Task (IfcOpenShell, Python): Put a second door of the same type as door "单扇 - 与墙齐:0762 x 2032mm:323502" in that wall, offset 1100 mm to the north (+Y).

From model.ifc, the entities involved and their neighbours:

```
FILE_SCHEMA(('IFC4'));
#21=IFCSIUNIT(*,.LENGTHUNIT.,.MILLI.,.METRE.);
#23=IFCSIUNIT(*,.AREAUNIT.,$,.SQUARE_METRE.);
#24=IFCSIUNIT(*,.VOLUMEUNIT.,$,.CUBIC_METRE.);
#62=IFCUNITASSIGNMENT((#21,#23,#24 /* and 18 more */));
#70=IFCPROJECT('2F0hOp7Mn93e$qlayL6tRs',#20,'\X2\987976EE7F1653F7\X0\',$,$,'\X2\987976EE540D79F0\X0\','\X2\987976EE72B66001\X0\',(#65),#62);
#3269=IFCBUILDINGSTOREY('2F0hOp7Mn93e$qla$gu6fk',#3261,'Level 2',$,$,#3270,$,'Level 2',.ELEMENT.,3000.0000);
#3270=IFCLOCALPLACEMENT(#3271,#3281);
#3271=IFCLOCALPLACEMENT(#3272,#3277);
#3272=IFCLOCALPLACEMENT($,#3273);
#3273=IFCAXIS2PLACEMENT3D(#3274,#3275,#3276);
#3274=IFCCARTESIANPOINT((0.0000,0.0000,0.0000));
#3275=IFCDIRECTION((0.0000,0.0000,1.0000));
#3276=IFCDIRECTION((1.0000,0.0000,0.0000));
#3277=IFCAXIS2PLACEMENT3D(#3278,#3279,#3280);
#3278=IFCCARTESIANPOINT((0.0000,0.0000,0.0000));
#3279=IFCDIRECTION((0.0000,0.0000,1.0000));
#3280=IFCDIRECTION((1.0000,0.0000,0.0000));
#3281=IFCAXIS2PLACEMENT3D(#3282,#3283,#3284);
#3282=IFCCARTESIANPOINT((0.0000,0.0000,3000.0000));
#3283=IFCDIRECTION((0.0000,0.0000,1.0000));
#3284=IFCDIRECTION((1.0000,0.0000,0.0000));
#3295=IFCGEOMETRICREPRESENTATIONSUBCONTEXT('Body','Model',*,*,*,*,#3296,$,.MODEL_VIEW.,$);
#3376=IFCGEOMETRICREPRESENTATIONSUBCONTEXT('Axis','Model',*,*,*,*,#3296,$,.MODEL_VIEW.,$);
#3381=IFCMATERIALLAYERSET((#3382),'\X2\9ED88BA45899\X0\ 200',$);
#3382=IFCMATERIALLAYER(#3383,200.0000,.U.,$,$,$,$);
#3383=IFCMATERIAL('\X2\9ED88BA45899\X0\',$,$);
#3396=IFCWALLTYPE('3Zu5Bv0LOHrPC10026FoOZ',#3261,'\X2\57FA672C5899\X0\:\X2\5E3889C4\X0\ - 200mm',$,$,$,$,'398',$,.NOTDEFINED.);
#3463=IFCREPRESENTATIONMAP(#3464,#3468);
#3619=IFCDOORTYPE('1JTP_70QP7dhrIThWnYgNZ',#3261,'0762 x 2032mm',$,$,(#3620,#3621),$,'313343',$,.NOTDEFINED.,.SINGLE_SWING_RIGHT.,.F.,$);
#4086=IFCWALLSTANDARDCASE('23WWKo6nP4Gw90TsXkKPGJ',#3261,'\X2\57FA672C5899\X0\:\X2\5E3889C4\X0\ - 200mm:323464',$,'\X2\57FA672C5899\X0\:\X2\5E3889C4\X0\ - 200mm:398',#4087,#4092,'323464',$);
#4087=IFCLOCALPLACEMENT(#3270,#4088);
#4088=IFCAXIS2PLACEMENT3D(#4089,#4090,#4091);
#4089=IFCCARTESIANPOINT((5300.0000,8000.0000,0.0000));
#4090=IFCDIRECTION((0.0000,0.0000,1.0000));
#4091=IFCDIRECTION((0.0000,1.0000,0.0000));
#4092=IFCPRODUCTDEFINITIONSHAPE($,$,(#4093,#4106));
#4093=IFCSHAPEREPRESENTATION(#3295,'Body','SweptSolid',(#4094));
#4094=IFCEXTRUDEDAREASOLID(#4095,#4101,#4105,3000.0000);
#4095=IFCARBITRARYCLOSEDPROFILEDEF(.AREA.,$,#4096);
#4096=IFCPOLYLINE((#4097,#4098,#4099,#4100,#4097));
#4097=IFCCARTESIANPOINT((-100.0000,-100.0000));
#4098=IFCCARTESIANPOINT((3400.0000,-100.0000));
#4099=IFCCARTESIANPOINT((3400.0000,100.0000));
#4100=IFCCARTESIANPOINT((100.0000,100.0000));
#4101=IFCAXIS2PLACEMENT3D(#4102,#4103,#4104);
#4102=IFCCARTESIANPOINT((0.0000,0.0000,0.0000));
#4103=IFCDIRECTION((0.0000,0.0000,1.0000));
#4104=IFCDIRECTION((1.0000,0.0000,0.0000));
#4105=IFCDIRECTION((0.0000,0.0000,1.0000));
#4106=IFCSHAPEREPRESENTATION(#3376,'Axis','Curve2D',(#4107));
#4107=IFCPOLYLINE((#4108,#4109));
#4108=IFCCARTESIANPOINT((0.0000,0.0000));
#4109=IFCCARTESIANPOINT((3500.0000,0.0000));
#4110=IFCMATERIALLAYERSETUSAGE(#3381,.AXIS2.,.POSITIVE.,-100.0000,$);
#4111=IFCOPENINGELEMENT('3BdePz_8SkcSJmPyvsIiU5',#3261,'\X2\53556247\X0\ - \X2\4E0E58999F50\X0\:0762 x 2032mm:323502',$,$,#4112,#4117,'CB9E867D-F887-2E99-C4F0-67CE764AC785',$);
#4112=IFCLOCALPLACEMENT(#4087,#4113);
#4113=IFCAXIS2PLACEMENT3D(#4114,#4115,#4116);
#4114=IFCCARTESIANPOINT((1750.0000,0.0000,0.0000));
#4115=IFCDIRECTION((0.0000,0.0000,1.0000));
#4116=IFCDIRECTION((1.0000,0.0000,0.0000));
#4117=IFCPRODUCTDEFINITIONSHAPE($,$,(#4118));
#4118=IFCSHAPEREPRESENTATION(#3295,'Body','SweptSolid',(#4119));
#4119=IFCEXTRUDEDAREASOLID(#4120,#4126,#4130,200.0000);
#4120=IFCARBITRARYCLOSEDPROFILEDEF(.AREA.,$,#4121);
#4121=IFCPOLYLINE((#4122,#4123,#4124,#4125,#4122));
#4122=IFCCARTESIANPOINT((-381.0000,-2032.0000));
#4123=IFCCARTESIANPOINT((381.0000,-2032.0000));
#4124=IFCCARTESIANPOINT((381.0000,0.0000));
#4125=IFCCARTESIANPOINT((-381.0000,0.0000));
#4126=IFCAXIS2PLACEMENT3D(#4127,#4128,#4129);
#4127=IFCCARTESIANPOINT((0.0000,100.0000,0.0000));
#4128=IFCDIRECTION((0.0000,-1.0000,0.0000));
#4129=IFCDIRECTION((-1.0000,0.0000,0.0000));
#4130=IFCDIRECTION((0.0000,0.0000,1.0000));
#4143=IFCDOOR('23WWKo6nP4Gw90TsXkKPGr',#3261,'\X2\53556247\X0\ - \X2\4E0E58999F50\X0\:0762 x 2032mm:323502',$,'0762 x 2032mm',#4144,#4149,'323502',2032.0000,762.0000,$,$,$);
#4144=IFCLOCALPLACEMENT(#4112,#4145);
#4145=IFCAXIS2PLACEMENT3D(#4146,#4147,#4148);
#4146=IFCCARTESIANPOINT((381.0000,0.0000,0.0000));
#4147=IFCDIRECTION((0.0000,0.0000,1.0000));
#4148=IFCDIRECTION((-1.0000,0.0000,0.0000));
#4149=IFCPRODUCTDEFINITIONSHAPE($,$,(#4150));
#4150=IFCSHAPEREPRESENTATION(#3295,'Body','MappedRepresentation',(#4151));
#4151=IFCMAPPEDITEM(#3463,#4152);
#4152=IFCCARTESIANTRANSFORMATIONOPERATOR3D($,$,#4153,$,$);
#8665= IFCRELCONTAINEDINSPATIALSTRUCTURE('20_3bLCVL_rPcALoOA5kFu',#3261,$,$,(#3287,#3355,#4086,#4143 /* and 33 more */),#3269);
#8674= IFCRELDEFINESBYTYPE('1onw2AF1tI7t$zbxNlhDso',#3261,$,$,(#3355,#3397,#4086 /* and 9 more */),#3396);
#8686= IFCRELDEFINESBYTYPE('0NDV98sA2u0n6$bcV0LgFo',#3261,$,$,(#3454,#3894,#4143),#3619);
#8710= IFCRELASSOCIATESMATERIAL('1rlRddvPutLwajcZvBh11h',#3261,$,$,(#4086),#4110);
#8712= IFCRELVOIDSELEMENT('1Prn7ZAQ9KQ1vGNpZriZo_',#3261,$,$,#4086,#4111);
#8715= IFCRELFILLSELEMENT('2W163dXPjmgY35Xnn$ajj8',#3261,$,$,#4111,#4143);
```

```python
import ifcopenshell
import ifcopenshell.api.feature
import ifcopenshell.api.geometry
import ifcopenshell.api.root
import ifcopenshell.geom
import ifcopenshell.util.element
import ifcopenshell.util.placement
import ifcopenshell.util.shape
import ifcopenshell.util.unit

model = ifcopenshell.open("model.ifc")
unit_scale = ifcopenshell.util.unit.calculate_unit_scale(model)
settings = ifcopenshell.geom.settings()


def volume(element):
    """Net volume in cubic metres, openings subtracted."""
    shape = ifcopenshell.geom.create_shape(settings, element)
    return ifcopenshell.util.shape.get_volume(shape.geometry)


def reuse_history(source, copy):
    """copy_class also copies each property set's owner history, people and application; keep the originals."""
    for rel in copy.IsDefinedBy:
        if rel.is_a("IfcRelDefinesByProperties") and (history := rel.RelatingPropertyDefinition.OwnerHistory):
            rel.RelatingPropertyDefinition.OwnerHistory = source.OwnerHistory
            ifcopenshell.util.element.remove_deep2(model, history)


door = model.by_guid("23WWKo6nP4Gw90TsXkKPGr")
opening = door.FillsVoids[0].RelatingOpeningElement
wall = opening.VoidsElements[0].RelatingBuildingElement
before = volume(wall)
shift = ifcopenshell.util.placement.get_local_placement(wall.ObjectPlacement)[:3, 0] * 1.1 / unit_scale

# copy_class copies the void relationship, type, container and properties, but no geometry.
new_opening = ifcopenshell.api.root.copy_class(model, product=opening)
new_opening.Representation = ifcopenshell.util.element.copy_deep(
    model, opening.Representation, exclude=["IfcGeometricRepresentationContext", "IfcRepresentationMap"]
)
new_opening.Name = "单扇 - 与墙齐:0762 x 2032mm"
new_opening.Tag = None
new_door = ifcopenshell.api.root.copy_class(model, product=door)
new_door.Representation = ifcopenshell.util.element.copy_deep(
    model, door.Representation, exclude=["IfcGeometricRepresentationContext", "IfcRepresentationMap"]
)
new_door.Name = "单扇 - 与墙齐:0762 x 2032mm"
new_door.Tag = None
reuse_history(door, new_door)
ifcopenshell.api.feature.add_filling(model, opening=new_opening, element=new_door)

for old, new in ((opening, new_opening), (door, new_door)):
    matrix = ifcopenshell.util.placement.get_local_placement(old.ObjectPlacement)
    matrix[:3, 3] += shift
    ifcopenshell.api.geometry.edit_object_placement(model, product=new, matrix=matrix, is_si=False)

after = volume(wall)

print(f"wall volume {before:.3f} -> {after:.3f} m3")

model.write("model_rev.ifc")
```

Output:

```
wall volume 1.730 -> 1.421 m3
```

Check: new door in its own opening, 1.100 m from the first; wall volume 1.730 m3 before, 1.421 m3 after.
